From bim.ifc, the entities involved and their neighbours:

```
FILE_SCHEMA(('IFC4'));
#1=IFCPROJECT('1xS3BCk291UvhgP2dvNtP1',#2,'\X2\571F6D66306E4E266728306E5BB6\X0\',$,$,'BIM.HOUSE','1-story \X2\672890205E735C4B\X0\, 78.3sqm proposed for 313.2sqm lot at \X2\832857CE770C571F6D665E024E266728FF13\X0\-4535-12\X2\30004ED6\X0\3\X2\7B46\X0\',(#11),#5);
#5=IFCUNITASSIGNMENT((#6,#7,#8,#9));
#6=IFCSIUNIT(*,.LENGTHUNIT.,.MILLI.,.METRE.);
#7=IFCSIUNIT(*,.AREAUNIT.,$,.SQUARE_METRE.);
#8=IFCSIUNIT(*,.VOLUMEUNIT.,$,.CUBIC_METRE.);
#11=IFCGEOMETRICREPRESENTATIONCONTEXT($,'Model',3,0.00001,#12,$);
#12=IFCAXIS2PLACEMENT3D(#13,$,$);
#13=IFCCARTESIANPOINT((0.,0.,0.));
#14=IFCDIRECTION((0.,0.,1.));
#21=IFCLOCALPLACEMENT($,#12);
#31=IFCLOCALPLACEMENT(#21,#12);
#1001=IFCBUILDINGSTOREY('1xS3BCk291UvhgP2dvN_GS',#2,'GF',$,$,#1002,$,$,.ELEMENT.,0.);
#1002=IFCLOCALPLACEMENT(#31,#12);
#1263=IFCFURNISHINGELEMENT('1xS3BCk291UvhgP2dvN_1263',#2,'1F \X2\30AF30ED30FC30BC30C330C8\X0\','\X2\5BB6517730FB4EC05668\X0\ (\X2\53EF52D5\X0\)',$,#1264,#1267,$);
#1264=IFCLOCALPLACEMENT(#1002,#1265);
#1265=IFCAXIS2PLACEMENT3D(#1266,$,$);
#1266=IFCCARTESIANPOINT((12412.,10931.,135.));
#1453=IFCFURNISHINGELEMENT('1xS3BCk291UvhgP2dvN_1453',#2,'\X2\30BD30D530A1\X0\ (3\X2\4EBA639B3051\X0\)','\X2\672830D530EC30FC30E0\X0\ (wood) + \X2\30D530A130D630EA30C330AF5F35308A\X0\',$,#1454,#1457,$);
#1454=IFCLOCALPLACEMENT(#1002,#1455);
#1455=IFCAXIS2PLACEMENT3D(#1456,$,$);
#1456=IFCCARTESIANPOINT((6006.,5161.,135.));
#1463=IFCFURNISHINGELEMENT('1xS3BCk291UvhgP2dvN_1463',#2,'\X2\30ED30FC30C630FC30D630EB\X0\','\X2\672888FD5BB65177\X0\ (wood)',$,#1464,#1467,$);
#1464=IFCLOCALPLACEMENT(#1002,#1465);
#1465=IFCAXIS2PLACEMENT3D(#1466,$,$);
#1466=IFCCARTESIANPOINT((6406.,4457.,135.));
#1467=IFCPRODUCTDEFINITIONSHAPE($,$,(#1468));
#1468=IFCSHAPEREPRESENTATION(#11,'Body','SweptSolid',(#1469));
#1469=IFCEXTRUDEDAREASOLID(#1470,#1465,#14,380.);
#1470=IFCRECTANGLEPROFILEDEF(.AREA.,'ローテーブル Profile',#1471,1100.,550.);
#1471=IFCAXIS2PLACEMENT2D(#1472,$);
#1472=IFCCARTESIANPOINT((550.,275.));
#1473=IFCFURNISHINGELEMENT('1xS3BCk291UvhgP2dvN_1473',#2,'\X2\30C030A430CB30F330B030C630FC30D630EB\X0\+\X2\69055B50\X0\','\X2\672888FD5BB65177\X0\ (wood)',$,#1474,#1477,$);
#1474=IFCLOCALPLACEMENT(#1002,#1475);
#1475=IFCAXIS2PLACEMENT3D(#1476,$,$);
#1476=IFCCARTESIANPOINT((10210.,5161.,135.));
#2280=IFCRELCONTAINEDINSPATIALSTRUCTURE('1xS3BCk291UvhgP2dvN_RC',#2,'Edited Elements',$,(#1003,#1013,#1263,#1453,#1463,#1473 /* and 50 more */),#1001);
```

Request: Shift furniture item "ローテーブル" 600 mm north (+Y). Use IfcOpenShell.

```python
import ifcopenshell
import ifcopenshell.api.geometry
import ifcopenshell.util.placement

model = ifcopenshell.open("bim.ifc")

item = model.by_guid("1xS3BCk291UvhgP2dvN_1463")
matrix = ifcopenshell.util.placement.get_local_placement(item.ObjectPlacement)
matrix[1, 3] += 600.0
ifcopenshell.api.geometry.edit_object_placement(model, product=item, matrix=matrix, is_si=False)

print(ifcopenshell.util.placement.get_local_placement(item.ObjectPlacement).round(3) + 0.0)

model.write("bim_edited.ifc")
```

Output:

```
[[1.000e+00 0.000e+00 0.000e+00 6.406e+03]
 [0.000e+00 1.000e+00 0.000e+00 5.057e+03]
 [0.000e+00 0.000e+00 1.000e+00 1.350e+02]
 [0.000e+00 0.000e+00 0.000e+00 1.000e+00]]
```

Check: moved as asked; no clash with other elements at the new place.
